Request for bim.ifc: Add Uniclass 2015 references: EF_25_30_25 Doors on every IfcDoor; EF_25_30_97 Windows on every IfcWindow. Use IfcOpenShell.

First a look at what the model holds.

```python
import ifcopenshell

model = ifcopenshell.open("bim.ifc")
print(model.schema)
print("classifications:", [c.Name for c in model.by_type("IfcClassification")])
for ifc_class in ("IfcDoor", "IfcRoof", "IfcStair", "IfcWall", "IfcWindow"):
    print(ifc_class, len(model.by_type(ifc_class)))
```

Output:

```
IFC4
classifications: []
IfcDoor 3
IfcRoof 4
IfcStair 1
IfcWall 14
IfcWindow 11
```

```python
import ifcopenshell
import ifcopenshell.api.classification

model = ifcopenshell.open("bim.ifc")

system = ifcopenshell.api.classification.add_classification(model, classification="Uniclass 2015")

codes = {
    "IfcDoor": ("EF_25_30_25", "Doors"),
    "IfcWindow": ("EF_25_30_97", "Windows"),
}
for ifc_class, (code, name) in codes.items():
    products = model.by_type(ifc_class)
    ifcopenshell.api.classification.add_reference(
        model, products=products, classification=system, identification=code, name=name
    )
    print(code, len(products))

model.write("bim_edited.ifc")
```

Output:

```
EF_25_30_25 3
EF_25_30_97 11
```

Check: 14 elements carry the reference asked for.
